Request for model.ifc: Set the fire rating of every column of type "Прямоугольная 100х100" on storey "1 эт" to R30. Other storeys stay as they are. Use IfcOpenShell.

First a look at what the model holds.

```python
import ifcopenshell
import ifcopenshell.util.element

model = ifcopenshell.open("model.ifc")
print(model.schema)
storey = next(s for s in model.by_type("IfcBuildingStorey") if s.Name == "1 эт")
columns = [e for e in ifcopenshell.util.element.get_decomposition(storey) if e.is_a("IfcColumn")]
seen = {}
for e in columns:
    element_type = ifcopenshell.util.element.get_type(e)
    key = (element_type.Name if element_type != e and element_type else None, ifcopenshell.util.element.get_pset(e, "Pset_ColumnCommon", "FireRating"))
    seen[key] = seen.get(key, 0) + 1
for (name, value), count in sorted(seen.items(), key=str):
    print(count, "x", name, "|", value)
```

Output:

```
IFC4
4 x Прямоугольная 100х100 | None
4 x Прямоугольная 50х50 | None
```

```python
import ifcopenshell
import ifcopenshell.api.pset
import ifcopenshell.util.element

model = ifcopenshell.open("model.ifc")

storey = next(s for s in model.by_type("IfcBuildingStorey") if s.Name == "1 эт")
columns = [e for e in ifcopenshell.util.element.get_decomposition(storey) if e.is_a("IfcColumn")]

count = 0
for e in columns:
    element_type = ifcopenshell.util.element.get_type(e)
    if element_type in (None, e) or element_type.Name != "Прямоугольная 100х100":
        continue
    # add_pset returns the element's existing set when there is one.
    pset = ifcopenshell.api.pset.add_pset(model, product=e, name="Pset_ColumnCommon")
    ifcopenshell.api.pset.edit_pset(model, pset=pset, properties={"FireRating": "R30"})
    count += 1

print(count, "columns updated")

model.write("model_rev.ifc")
```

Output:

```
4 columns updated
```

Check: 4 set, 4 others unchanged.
